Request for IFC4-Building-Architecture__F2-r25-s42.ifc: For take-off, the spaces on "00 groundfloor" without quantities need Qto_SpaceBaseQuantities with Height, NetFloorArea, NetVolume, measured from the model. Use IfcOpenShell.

First a look at what the model holds.

```python
import ifcopenshell
import ifcopenshell.util.element
import ifcopenshell.util.unit

model = ifcopenshell.open("IFC4-Building-Architecture__F2-r25-s42.ifc")
print(model.schema)
for unit_type in ("LENGTHUNIT", "AREAUNIT", "VOLUMEUNIT"):
    print(unit_type, ifcopenshell.util.unit.calculate_unit_scale(model, unit_type))
storey = next(s for s in model.by_type("IfcBuildingStorey") if s.Name == "00 groundfloor")
spaces = [e for e in ifcopenshell.util.element.get_decomposition(storey) if e.is_a("IfcSpace")]
for e in sorted(spaces, key=lambda e: e.id()):
    print(e.id(), e.is_a(), e.Name, list(ifcopenshell.util.element.get_psets(e, qtos_only=True)), sep=" | ")
```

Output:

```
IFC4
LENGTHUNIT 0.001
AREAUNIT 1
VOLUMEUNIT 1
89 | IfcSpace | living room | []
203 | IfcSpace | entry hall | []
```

```python
import ifcopenshell
import ifcopenshell.api.pset
import ifcopenshell.geom
import ifcopenshell.util.element
import ifcopenshell.util.shape
import ifcopenshell.util.unit

model = ifcopenshell.open("IFC4-Building-Architecture__F2-r25-s42.ifc")
unit_scale = ifcopenshell.util.unit.calculate_unit_scale(model)
area_scale = ifcopenshell.util.unit.calculate_unit_scale(model, "AREAUNIT")
volume_scale = ifcopenshell.util.unit.calculate_unit_scale(model, "VOLUMEUNIT")
settings = ifcopenshell.geom.settings()

storey = next(s for s in model.by_type("IfcBuildingStorey") if s.Name == "00 groundfloor")
spaces = [e for e in ifcopenshell.util.element.get_decomposition(storey) if e.is_a("IfcSpace")]

for e in sorted(spaces, key=lambda e: e.id()):
    if ifcopenshell.util.element.get_psets(e, qtos_only=True, should_inherit=False):
        continue
    # Geometry comes back in metres, in the element's own axes.
    shape = ifcopenshell.geom.create_shape(settings, e)
    values = {
        "Height": ifcopenshell.util.shape.get_z(shape.geometry) / unit_scale,
        "NetFloorArea": ifcopenshell.util.shape.get_footprint_area(shape.geometry) / area_scale,
        "NetVolume": ifcopenshell.util.shape.get_volume(shape.geometry) / volume_scale,
    }
    qto = ifcopenshell.api.pset.add_qto(model, product=e, name="Qto_SpaceBaseQuantities")
    ifcopenshell.api.pset.edit_qto(model, qto=qto, properties=values)
    print(e.id(), {k: round(v, 3) for k, v in values.items()})

model.write("IFC4-Building-Architecture__F2-r25-s42_updated.ifc")
```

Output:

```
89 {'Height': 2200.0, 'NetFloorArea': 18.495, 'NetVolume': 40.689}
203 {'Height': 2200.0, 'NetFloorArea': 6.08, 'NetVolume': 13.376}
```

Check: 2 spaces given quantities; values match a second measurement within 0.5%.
